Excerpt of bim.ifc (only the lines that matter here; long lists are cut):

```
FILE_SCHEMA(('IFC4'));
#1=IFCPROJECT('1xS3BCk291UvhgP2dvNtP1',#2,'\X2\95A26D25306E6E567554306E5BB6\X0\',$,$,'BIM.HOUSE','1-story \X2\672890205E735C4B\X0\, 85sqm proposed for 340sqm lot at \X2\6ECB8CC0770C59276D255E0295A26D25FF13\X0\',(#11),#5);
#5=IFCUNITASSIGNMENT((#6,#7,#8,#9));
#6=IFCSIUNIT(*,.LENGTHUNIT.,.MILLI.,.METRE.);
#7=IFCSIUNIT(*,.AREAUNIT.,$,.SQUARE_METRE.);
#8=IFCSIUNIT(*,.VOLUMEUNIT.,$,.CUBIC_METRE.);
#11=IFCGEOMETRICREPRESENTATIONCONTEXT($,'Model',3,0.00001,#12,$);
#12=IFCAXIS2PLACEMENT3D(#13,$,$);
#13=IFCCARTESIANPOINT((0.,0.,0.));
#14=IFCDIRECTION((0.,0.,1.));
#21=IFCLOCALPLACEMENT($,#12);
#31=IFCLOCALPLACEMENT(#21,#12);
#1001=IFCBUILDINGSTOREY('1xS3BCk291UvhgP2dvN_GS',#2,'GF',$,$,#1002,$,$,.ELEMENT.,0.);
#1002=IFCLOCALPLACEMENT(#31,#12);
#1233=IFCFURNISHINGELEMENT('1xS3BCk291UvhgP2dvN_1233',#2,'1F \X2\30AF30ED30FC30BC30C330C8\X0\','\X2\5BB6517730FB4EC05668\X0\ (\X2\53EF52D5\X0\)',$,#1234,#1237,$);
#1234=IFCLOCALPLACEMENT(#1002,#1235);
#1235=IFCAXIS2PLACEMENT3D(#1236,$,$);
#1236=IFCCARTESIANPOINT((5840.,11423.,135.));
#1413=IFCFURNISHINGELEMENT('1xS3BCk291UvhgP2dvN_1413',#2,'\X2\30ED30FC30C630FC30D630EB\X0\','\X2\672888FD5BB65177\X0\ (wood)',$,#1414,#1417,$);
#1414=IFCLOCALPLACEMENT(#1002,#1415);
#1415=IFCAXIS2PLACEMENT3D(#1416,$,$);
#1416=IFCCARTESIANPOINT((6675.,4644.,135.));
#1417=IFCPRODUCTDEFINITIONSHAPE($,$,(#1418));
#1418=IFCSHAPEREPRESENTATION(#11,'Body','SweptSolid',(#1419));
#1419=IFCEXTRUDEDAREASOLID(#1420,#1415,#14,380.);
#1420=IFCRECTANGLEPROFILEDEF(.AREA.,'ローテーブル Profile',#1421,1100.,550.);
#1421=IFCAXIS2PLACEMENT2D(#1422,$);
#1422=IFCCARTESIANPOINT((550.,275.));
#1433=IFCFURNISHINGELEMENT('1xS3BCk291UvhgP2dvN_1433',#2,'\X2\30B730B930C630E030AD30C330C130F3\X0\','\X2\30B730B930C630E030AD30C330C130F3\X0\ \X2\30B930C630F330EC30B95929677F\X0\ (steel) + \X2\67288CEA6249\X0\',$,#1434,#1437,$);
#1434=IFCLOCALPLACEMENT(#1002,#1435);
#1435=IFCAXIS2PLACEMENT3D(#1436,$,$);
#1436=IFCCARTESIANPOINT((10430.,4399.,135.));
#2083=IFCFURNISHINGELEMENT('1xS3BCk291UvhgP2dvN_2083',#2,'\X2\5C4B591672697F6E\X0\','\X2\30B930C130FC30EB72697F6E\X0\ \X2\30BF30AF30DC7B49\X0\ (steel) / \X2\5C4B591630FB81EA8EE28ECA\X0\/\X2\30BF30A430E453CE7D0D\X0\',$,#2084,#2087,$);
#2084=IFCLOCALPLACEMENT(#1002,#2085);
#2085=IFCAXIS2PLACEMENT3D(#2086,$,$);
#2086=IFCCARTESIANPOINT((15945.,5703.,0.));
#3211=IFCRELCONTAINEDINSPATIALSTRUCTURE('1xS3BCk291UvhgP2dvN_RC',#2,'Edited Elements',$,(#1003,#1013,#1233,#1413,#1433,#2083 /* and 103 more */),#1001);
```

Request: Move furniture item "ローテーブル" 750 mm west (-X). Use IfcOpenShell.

```python
import ifcopenshell
import ifcopenshell.api.geometry
import ifcopenshell.util.placement
import ifcopenshell.util.unit

model = ifcopenshell.open("bim.ifc")
unit_scale = ifcopenshell.util.unit.calculate_unit_scale(model)

item = model.by_guid("1xS3BCk291UvhgP2dvN_1413")
matrix = ifcopenshell.util.placement.get_local_placement(item.ObjectPlacement)
matrix[0, 3] -= 0.75 / unit_scale
ifcopenshell.api.geometry.edit_object_placement(model, product=item, matrix=matrix, is_si=False)

print(ifcopenshell.util.placement.get_local_placement(item.ObjectPlacement).round(3) + 0.0)

model.write("bim_rev.ifc")
```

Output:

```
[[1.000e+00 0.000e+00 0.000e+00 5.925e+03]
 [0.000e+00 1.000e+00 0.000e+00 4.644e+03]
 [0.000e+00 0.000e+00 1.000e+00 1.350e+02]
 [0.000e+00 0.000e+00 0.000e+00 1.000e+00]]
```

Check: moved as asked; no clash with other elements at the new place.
